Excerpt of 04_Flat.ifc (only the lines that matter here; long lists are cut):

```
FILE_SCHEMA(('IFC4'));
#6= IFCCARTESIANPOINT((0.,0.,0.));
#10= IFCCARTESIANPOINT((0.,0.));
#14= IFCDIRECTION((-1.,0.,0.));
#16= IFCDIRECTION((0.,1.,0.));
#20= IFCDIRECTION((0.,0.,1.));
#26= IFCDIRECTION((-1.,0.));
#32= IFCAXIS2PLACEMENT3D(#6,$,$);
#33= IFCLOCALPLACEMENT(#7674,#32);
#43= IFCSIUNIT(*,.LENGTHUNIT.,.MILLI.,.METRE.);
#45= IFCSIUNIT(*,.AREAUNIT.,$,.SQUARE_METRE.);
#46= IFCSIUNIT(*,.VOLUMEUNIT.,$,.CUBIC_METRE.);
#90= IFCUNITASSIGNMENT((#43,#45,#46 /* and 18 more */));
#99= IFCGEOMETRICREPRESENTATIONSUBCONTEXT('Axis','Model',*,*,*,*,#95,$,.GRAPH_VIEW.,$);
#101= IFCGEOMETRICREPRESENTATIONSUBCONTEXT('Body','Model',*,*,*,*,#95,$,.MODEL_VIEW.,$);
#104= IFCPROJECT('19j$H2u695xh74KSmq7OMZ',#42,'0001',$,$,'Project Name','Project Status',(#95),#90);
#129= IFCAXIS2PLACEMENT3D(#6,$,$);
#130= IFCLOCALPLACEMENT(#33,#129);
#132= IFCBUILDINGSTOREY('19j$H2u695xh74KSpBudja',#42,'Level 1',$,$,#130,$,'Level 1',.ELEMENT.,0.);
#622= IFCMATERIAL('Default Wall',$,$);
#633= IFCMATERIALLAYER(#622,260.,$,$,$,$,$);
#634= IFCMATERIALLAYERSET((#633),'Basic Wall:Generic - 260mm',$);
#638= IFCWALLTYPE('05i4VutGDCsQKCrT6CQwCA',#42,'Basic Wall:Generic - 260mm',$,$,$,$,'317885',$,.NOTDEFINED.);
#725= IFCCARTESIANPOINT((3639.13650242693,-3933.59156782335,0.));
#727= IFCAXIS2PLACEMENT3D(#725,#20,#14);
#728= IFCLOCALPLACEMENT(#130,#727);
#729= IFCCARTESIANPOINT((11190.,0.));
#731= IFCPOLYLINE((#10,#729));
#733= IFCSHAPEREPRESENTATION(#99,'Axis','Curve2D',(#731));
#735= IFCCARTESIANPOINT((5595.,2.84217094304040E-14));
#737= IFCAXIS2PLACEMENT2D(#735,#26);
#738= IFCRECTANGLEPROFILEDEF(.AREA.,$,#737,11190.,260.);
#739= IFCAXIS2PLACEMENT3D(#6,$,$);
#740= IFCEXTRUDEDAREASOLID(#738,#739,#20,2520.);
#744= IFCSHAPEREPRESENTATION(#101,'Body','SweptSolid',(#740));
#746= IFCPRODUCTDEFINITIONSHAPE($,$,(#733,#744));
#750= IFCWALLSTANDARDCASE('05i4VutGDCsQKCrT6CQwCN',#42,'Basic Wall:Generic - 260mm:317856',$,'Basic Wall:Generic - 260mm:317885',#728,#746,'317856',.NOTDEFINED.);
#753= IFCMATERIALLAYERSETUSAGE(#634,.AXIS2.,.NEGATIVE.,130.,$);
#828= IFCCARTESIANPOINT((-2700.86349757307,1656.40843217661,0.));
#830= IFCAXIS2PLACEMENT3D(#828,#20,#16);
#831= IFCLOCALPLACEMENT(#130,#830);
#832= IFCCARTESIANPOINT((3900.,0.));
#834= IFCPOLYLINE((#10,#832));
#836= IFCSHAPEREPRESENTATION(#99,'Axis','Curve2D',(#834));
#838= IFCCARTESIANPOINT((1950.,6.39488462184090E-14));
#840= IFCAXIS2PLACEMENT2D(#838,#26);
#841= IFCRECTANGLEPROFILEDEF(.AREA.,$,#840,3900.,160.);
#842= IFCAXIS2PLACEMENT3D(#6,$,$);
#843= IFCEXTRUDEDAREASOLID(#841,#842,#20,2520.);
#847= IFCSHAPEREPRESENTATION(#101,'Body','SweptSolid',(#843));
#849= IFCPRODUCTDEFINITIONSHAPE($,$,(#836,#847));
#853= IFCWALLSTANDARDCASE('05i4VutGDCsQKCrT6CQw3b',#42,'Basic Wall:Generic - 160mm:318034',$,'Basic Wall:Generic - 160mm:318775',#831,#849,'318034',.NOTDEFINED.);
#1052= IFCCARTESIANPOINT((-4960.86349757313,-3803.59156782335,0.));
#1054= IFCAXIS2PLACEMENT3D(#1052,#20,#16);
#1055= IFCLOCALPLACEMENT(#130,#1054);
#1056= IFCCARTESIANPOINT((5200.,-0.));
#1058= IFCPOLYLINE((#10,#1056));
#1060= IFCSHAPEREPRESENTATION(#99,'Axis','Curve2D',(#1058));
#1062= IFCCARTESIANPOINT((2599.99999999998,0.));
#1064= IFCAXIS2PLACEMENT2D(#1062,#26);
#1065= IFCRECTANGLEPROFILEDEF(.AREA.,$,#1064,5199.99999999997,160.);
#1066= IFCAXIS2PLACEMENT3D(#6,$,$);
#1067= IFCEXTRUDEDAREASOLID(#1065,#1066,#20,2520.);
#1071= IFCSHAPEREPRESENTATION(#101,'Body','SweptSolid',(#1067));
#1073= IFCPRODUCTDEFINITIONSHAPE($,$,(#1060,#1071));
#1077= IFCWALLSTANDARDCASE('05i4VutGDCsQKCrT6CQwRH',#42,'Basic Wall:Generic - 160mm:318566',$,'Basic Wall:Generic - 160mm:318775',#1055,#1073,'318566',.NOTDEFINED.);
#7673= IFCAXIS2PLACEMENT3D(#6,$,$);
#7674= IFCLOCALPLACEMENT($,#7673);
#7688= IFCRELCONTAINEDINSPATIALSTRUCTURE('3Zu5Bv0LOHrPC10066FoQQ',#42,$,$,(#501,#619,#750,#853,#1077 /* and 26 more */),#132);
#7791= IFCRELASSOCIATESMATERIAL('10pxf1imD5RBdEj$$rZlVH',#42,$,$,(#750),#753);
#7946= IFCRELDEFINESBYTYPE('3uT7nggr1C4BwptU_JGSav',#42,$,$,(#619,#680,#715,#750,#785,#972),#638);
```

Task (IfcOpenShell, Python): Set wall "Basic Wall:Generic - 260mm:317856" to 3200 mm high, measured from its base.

```python
import ifcopenshell
import ifcopenshell.geom
import ifcopenshell.util.representation
import ifcopenshell.util.shape
import ifcopenshell.util.unit

model = ifcopenshell.open("04_Flat.ifc")
unit_scale = ifcopenshell.util.unit.calculate_unit_scale(model)
settings = ifcopenshell.geom.settings()


def volume(element):
    """Net volume in cubic metres, openings subtracted."""
    shape = ifcopenshell.geom.create_shape(settings, element)
    return ifcopenshell.util.shape.get_volume(shape.geometry)


wall = model.by_guid("05i4VutGDCsQKCrT6CQwCN")
before = volume(wall)

body = ifcopenshell.util.representation.get_representation(wall, "Model", "Body")
solid = body.Items[0]
old_height = solid.Depth
solid.Depth = 3.2 / unit_scale
after = volume(wall)

print(f"height {old_height:g} -> {solid.Depth:g}, volume {before:.3f} -> {after:.3f} m3")

model.write("04_Flat_updated.ifc")
```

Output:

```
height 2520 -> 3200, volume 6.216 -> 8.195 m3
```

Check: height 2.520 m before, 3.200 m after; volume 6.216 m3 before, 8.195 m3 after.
